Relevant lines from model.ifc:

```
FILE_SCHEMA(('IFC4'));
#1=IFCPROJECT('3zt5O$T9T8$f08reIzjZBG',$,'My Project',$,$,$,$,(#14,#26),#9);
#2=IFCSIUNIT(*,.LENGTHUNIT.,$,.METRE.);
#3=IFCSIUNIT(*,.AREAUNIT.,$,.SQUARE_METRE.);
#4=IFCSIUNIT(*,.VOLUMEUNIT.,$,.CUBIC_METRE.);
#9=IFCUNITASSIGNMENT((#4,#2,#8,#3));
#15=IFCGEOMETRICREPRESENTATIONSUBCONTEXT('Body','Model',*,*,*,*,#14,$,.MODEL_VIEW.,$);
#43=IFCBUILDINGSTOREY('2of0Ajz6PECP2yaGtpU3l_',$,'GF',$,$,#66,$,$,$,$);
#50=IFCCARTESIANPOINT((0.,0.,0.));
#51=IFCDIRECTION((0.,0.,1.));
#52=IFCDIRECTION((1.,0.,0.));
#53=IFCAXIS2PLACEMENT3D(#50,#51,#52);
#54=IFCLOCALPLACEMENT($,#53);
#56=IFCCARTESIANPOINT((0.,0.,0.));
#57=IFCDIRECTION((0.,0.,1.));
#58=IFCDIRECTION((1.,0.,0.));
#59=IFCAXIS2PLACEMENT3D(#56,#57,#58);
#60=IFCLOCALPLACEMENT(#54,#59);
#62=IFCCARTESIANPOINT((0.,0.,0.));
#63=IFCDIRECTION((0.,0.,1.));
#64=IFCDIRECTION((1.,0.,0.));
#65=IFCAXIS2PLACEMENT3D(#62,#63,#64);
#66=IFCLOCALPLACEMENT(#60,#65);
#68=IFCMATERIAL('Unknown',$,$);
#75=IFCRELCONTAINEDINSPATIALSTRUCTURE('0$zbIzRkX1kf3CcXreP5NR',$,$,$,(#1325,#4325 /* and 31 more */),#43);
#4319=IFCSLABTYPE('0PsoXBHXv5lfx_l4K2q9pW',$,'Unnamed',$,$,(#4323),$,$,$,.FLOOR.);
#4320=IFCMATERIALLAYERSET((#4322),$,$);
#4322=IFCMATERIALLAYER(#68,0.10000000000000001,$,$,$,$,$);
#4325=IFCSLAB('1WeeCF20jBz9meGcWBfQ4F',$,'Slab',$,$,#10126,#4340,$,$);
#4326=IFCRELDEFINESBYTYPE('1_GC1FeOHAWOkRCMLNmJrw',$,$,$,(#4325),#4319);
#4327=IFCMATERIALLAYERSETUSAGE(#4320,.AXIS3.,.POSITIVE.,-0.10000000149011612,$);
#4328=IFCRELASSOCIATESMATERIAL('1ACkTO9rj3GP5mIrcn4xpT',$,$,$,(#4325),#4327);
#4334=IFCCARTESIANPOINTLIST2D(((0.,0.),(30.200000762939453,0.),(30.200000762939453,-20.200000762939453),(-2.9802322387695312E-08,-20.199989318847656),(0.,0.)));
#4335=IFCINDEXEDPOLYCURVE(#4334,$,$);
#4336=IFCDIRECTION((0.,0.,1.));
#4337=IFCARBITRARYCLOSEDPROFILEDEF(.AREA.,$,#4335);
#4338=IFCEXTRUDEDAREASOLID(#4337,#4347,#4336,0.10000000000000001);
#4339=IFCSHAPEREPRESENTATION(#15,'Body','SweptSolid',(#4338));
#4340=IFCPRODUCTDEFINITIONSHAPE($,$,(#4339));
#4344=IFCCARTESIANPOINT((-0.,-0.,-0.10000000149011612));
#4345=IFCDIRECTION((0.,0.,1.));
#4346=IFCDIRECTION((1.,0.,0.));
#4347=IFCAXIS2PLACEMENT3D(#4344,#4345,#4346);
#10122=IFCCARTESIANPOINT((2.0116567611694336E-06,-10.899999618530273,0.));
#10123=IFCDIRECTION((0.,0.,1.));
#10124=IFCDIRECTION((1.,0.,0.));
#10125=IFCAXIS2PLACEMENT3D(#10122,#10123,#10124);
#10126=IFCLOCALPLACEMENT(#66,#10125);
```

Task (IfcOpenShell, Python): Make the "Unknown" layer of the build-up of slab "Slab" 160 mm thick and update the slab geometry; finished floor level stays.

```python
import ifcopenshell
import ifcopenshell.util.element
import ifcopenshell.util.representation
import ifcopenshell.util.unit

model = ifcopenshell.open("model.ifc")
unit_scale = ifcopenshell.util.unit.calculate_unit_scale(model)

layer_set = model.by_id(4320)
layer = next(l for l in layer_set.MaterialLayers if l.Material and l.Material.Name == "Unknown")
change = 0.16 / unit_scale - layer.LayerThickness
layer.LayerThickness += change

# Geometry does not follow the layer set by itself.
slabs = [e for e in ifcopenshell.util.element.get_elements_by_material(model, layer_set) if e.is_a("IfcSlab")]
for slab in sorted(slabs, key=lambda e: e.id()):
    body = ifcopenshell.util.representation.get_representation(slab, "Model", "Body")
    solid = body.Items[0]
    old_depth = solid.Depth
    solid.Depth += change
    # Extruded upwards: lower the start of the extrusion so the top stays.
    x, y, z = solid.Position.Location.Coordinates
    solid.Position.Location = model.createIfcCartesianPoint((x, y, z - change))
    print(slab.id(), f"{old_depth:g} -> {solid.Depth:g}")

# The layers are counted up from the underside, which has moved.
for usage in {ifcopenshell.util.element.get_material(slab) for slab in slabs}:
    usage.OffsetFromReferenceLine -= change

model.write("model_edited.ifc")
```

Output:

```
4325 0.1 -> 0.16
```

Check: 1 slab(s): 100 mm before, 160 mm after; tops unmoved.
